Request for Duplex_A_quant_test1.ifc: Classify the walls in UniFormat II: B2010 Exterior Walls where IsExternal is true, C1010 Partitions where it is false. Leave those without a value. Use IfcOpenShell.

First a look at what the model holds.

```python
import ifcopenshell
import ifcopenshell.util.element

model = ifcopenshell.open("Duplex_A_quant_test1.ifc")
print(model.schema)
print("classifications:", [c.Name for c in model.by_type("IfcClassification")])
values = [ifcopenshell.util.element.get_pset(e, "Pset_WallCommon", "IsExternal") for e in model.by_type("IfcWall")]
for value in (True, False, None):
    print("IsExternal", value, values.count(value))
```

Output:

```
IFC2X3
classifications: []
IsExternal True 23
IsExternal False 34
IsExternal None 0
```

```python
import ifcopenshell
import ifcopenshell.api.classification
import ifcopenshell.util.element

model = ifcopenshell.open("Duplex_A_quant_test1.ifc")

# IFC2X3 requires Source and Edition and has no link from the project to the system.
system = model.create_entity("IfcClassification", Source="ASTM", Edition="E1557", Name="UniFormat II")

walls = model.by_type("IfcWall")
external = {e: ifcopenshell.util.element.get_pset(e, "Pset_WallCommon", "IsExternal") for e in walls}
for flag, code, name in ((True, "B2010", "Exterior Walls"), (False, "C1010", "Partitions")):
    products = [e for e in walls if external[e] is flag]
    ifcopenshell.api.classification.add_reference(
        model, products=products, classification=system, identification=code, name=name
    )
    print(code, len(products))

model.write("Duplex_A_quant_test1_updated.ifc")
```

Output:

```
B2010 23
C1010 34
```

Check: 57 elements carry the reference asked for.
